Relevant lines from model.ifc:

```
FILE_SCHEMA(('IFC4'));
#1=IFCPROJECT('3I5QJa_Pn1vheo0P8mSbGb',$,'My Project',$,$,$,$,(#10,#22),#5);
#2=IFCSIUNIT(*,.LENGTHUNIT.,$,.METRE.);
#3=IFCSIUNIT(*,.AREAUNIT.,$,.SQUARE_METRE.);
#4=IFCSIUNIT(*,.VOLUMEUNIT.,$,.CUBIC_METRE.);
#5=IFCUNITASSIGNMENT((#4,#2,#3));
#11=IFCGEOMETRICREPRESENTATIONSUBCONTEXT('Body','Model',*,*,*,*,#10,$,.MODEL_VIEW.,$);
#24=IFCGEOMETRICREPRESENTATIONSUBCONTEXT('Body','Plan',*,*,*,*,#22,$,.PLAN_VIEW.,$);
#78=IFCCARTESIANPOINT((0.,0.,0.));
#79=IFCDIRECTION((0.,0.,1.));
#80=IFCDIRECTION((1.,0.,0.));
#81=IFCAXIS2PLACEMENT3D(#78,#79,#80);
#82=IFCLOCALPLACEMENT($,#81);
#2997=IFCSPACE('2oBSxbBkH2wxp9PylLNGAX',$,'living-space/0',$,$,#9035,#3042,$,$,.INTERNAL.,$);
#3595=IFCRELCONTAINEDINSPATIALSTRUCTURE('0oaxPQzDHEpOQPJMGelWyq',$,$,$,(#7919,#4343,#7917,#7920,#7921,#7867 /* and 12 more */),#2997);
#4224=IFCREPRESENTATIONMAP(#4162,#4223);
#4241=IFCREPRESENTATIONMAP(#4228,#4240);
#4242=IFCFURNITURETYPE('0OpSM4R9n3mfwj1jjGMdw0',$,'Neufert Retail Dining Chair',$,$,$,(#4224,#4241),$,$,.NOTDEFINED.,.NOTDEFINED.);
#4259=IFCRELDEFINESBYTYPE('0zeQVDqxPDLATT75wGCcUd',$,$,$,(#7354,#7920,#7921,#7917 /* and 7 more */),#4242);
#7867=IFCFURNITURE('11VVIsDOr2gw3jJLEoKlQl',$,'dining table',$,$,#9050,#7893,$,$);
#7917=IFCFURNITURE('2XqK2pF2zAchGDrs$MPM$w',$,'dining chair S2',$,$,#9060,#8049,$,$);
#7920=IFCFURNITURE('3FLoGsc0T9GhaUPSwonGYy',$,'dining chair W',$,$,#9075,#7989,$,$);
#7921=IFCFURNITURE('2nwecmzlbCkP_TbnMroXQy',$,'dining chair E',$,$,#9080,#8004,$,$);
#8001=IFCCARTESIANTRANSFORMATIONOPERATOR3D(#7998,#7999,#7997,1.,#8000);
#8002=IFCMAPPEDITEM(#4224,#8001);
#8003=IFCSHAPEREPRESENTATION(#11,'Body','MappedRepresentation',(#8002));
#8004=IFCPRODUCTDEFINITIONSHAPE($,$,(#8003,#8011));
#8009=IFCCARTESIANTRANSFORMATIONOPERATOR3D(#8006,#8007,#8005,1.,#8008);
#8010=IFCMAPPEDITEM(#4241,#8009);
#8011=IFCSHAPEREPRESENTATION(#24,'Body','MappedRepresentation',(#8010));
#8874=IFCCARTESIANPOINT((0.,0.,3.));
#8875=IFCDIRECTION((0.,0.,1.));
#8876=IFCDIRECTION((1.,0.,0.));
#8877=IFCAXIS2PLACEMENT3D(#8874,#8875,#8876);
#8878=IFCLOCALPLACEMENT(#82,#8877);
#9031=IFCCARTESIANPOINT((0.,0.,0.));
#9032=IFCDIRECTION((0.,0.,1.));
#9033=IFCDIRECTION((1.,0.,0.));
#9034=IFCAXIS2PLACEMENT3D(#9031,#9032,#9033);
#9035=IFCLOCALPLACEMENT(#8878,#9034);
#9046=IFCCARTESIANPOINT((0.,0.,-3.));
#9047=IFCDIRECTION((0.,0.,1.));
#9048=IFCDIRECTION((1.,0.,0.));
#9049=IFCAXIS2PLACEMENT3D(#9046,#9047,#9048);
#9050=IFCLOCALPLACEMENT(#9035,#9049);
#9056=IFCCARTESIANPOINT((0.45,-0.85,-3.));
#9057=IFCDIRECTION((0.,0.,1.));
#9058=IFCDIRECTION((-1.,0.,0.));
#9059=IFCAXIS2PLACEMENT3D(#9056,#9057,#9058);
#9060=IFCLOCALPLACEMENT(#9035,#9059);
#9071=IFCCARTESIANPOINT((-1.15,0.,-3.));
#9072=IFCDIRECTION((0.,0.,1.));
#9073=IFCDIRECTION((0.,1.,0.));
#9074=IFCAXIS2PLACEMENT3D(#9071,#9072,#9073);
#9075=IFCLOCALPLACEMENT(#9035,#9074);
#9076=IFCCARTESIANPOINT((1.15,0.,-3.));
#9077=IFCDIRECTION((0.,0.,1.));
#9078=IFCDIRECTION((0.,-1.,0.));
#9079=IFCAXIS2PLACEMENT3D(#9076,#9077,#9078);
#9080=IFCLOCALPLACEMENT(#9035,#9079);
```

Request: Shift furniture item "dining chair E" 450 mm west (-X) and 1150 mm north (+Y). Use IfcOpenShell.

```python
import ifcopenshell
import ifcopenshell.api.geometry
import ifcopenshell.util.placement
import ifcopenshell.util.unit

model = ifcopenshell.open("model.ifc")
unit_scale = ifcopenshell.util.unit.calculate_unit_scale(model)

item = model.by_id(7921)
matrix = ifcopenshell.util.placement.get_local_placement(item.ObjectPlacement)
matrix[0, 3] -= 0.45 / unit_scale
matrix[1, 3] += 1.15 / unit_scale
ifcopenshell.api.geometry.edit_object_placement(model, product=item, matrix=matrix, is_si=False)

print(ifcopenshell.util.placement.get_local_placement(item.ObjectPlacement).round(3) + 0.0)

model.write("model_edited.ifc")
```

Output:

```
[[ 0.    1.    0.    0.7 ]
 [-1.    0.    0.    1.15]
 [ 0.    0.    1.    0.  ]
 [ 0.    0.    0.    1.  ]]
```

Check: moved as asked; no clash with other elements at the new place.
